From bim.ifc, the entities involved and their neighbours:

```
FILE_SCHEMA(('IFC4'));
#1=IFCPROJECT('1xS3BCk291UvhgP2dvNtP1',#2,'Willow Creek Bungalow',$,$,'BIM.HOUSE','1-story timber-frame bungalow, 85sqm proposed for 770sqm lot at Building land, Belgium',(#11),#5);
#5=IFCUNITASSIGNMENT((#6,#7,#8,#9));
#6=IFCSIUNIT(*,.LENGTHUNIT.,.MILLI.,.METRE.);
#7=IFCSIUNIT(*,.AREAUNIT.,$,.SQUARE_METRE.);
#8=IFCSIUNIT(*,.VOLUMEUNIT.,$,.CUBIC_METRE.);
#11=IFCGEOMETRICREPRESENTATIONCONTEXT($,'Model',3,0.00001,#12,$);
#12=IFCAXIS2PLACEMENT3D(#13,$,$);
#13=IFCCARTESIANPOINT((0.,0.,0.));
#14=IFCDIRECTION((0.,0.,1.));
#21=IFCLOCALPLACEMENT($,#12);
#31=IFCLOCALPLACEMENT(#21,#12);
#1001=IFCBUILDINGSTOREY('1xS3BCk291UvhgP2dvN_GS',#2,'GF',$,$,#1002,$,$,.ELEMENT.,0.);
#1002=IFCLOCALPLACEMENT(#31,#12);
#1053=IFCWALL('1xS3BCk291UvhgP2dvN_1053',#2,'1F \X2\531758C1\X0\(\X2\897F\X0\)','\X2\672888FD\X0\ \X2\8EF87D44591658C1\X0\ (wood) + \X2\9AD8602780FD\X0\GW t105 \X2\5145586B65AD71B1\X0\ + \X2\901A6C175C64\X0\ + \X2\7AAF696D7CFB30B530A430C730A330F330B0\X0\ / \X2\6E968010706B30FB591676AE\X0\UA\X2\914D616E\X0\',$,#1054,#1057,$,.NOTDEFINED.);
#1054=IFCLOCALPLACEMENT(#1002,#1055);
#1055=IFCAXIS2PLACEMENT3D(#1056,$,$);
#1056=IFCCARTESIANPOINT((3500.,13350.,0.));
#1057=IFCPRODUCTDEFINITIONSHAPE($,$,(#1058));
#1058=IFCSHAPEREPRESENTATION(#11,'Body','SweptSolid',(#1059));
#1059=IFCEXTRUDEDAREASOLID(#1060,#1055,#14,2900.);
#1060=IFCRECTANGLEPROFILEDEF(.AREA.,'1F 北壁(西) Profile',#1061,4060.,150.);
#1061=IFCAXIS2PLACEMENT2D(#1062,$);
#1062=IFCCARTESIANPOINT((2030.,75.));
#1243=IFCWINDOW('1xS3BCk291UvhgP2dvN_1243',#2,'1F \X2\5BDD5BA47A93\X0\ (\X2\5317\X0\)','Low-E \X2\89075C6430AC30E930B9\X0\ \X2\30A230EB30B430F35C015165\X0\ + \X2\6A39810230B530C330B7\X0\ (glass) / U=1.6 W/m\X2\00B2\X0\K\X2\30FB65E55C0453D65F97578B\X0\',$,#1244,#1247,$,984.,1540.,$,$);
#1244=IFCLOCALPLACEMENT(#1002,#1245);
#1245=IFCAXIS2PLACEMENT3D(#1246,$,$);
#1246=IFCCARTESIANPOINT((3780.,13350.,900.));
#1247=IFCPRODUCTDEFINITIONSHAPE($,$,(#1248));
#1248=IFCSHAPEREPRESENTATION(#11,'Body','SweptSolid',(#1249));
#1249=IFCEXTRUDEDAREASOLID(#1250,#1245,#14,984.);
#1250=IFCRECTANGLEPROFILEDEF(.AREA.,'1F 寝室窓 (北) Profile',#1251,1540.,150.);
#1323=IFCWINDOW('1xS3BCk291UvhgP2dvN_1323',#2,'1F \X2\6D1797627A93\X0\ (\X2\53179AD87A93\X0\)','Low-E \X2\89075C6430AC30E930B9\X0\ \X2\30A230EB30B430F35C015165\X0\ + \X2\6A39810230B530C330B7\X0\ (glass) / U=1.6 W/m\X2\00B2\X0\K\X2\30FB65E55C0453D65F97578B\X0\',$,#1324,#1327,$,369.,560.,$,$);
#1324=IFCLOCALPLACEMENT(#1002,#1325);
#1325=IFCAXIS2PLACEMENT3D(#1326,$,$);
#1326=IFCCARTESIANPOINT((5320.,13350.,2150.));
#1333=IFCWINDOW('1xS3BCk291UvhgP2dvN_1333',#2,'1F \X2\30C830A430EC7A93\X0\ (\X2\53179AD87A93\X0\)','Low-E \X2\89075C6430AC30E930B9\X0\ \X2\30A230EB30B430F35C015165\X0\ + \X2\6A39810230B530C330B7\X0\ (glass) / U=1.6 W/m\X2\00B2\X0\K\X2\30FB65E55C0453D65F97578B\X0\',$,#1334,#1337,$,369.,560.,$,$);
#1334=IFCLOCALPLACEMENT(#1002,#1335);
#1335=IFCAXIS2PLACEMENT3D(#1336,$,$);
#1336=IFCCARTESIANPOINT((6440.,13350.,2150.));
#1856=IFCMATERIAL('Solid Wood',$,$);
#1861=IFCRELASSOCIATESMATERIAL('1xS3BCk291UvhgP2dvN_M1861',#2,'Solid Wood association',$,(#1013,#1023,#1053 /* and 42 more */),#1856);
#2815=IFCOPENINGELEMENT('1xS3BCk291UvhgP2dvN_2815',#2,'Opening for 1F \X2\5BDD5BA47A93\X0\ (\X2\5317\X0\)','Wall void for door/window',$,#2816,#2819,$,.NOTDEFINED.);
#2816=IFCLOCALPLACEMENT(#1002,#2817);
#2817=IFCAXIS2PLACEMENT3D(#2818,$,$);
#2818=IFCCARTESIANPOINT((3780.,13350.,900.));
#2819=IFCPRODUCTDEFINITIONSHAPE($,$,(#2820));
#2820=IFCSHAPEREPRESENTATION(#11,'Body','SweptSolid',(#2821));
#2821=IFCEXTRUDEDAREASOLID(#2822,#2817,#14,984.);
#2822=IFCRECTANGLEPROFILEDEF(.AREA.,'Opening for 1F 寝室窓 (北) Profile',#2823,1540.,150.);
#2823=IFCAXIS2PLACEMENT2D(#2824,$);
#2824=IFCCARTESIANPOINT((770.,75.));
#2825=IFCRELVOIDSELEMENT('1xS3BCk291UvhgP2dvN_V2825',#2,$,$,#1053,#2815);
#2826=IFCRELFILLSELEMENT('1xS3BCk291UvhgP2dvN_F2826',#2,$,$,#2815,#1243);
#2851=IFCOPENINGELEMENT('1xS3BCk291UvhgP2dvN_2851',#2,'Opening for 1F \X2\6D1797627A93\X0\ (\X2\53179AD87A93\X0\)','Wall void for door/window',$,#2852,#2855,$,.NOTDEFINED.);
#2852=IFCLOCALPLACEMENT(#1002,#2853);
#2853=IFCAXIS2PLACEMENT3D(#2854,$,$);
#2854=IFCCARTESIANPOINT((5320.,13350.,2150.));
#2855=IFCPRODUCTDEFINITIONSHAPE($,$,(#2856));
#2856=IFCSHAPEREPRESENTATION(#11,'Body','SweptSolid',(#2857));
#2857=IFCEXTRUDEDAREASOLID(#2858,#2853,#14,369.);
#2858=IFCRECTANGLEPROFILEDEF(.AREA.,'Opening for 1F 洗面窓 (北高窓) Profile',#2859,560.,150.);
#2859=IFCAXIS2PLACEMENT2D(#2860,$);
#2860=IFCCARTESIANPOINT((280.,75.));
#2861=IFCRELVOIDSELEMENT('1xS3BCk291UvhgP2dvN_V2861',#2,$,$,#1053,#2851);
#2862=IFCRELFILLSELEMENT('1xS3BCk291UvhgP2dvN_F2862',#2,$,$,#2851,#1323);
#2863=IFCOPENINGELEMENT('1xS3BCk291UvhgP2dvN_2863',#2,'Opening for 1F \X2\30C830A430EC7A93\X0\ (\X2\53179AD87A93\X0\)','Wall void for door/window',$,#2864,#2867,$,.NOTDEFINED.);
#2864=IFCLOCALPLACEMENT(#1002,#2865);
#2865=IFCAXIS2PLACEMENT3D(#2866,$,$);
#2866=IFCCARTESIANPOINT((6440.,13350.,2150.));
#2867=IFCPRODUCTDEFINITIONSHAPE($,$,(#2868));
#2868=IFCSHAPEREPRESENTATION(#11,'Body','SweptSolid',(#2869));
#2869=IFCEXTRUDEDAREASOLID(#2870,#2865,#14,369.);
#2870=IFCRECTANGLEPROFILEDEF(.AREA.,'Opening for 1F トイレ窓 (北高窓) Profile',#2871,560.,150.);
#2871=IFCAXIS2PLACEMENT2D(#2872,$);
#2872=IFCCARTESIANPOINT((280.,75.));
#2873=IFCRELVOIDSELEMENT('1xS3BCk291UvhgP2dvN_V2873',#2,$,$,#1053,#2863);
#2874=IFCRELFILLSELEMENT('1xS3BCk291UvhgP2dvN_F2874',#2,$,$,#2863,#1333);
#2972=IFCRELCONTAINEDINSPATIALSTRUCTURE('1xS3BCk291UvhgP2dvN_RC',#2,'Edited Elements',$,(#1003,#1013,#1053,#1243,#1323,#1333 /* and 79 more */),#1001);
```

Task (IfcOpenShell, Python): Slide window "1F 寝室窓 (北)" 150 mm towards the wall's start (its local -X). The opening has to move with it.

```python
import ifcopenshell
import ifcopenshell.api.geometry
import ifcopenshell.util.placement
import ifcopenshell.util.unit

model = ifcopenshell.open("bim.ifc")
unit_scale = ifcopenshell.util.unit.calculate_unit_scale(model)

window = model.by_guid("1xS3BCk291UvhgP2dvN_1243")
opening = window.FillsVoids[0].RelatingOpeningElement
wall = opening.VoidsElements[0].RelatingBuildingElement

wall_matrix = ifcopenshell.util.placement.get_local_placement(wall.ObjectPlacement)
shift = wall_matrix[:3, 0] * -0.15 / unit_scale
before = ifcopenshell.util.placement.get_local_placement(window.ObjectPlacement)[:3, 3].copy()

# The window is not placed relative to its opening, so move both.
for product in (opening, window):
    matrix = ifcopenshell.util.placement.get_local_placement(product.ObjectPlacement)
    matrix[:3, 3] += shift
    ifcopenshell.api.geometry.edit_object_placement(model, product=product, matrix=matrix, is_si=False)

after = ifcopenshell.util.placement.get_local_placement(window.ObjectPlacement)[:3, 3]
print("window moved by", (after - before).round(3) + 0.0)

model.write("bim_rev.ifc")
```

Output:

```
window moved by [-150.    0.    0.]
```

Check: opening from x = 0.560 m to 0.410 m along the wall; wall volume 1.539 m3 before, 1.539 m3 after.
